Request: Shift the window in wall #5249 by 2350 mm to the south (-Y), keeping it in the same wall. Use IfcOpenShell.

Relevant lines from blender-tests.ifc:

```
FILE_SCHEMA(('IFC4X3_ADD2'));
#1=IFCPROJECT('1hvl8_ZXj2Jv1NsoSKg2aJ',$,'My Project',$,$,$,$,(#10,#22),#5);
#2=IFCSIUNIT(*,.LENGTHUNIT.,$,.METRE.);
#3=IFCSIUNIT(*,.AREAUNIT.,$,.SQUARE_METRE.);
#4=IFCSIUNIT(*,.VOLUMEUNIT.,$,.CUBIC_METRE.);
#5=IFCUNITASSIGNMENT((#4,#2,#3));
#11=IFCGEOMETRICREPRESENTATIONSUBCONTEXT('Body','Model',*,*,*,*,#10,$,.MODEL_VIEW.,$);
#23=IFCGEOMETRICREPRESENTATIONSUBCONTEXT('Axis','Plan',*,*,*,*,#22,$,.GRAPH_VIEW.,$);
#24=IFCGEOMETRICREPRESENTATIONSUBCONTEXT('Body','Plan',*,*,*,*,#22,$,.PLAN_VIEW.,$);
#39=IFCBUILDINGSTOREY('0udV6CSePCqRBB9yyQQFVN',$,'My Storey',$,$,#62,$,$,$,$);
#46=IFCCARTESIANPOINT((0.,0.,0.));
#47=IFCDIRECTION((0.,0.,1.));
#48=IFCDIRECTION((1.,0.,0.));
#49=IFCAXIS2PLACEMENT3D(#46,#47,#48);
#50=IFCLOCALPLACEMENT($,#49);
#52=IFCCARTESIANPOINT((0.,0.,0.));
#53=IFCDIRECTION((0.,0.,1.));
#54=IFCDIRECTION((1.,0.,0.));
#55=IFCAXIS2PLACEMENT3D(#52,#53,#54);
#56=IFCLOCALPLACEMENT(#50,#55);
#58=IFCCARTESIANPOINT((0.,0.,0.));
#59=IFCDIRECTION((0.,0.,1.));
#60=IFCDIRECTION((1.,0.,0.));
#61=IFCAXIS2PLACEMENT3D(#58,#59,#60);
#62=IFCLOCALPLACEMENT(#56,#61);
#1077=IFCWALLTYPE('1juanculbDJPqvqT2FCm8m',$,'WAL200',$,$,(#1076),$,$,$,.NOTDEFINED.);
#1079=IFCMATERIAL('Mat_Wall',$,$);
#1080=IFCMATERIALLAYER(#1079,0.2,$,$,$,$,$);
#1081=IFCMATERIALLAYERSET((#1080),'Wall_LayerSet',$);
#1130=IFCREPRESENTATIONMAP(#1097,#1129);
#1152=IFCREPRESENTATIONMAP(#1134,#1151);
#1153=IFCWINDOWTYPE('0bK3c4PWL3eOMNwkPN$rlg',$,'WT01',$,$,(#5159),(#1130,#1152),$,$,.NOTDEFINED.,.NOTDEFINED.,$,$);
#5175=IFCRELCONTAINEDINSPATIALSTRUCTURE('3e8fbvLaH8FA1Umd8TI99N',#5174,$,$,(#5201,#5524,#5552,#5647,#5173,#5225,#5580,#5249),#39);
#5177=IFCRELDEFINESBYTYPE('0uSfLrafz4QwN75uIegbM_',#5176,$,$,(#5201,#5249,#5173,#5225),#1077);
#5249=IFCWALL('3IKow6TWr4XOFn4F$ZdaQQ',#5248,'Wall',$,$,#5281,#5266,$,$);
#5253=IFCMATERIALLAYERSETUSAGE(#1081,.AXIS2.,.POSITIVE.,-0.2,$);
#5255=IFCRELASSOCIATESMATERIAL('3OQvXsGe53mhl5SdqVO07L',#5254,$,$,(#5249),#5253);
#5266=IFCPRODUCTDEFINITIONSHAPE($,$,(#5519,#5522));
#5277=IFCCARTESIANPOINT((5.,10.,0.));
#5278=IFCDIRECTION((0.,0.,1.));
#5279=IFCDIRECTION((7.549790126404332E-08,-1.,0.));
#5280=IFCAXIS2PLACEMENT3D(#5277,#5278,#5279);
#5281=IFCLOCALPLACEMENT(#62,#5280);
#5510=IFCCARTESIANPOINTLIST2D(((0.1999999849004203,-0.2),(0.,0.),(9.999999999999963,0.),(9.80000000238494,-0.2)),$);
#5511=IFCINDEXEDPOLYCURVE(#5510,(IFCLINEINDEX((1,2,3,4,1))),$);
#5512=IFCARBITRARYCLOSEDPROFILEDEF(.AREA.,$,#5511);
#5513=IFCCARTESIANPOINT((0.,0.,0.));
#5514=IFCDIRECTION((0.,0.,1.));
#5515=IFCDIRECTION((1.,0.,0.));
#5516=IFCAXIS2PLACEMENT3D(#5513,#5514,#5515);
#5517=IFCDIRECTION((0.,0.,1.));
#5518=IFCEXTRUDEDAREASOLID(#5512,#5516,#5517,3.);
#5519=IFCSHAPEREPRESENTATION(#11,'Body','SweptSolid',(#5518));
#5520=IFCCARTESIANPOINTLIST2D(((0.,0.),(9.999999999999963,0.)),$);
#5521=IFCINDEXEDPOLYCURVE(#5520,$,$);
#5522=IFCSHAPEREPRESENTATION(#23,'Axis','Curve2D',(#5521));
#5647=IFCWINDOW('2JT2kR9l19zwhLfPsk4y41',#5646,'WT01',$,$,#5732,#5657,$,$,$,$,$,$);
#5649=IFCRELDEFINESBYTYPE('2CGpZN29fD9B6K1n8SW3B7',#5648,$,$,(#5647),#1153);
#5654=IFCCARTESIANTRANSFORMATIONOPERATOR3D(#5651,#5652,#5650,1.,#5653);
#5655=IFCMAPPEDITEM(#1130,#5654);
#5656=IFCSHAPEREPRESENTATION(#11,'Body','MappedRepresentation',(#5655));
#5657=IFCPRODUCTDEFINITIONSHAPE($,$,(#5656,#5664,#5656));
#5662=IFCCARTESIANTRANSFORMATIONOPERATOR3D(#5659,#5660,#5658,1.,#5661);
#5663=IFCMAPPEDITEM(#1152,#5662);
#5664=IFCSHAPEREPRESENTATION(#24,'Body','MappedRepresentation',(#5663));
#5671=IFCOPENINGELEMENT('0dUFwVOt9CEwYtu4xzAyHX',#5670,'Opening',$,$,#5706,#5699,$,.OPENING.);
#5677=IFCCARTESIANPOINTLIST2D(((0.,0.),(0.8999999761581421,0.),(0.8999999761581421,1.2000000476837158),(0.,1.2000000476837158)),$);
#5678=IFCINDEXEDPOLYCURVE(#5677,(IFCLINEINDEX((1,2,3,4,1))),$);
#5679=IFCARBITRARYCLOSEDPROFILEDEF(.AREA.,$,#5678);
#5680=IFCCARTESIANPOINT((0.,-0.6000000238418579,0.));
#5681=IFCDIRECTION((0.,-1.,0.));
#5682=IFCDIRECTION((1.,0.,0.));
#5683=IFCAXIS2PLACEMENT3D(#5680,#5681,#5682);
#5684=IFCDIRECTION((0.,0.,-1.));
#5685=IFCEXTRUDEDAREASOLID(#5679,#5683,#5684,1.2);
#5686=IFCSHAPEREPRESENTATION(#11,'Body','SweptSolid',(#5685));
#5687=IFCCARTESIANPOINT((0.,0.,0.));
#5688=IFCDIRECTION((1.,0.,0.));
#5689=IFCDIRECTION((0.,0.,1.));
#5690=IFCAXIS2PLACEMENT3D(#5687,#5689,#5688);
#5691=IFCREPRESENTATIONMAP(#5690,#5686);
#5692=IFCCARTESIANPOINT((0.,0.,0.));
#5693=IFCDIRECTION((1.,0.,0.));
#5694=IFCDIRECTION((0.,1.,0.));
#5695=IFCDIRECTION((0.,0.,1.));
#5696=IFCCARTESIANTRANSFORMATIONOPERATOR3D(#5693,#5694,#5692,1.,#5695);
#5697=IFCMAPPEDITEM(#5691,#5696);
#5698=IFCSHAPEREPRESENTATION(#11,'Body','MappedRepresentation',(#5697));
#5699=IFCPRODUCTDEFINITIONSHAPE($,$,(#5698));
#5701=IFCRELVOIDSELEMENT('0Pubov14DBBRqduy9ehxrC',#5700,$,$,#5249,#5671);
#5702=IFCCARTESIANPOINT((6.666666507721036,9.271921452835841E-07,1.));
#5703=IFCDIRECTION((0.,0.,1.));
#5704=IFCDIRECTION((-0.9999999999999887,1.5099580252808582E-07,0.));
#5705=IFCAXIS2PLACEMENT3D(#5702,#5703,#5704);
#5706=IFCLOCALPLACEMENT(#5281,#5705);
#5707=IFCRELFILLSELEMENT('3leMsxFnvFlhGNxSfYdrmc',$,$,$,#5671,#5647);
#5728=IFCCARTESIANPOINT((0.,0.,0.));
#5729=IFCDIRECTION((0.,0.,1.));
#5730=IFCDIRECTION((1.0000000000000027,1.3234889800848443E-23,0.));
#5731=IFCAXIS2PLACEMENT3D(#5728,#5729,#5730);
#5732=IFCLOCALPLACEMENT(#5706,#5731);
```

```python
import ifcopenshell
import ifcopenshell.api.geometry
import ifcopenshell.util.placement

model = ifcopenshell.open("blender-tests.ifc")

window = model.by_id(5647)
opening = window.FillsVoids[0].RelatingOpeningElement
wall = opening.VoidsElements[0].RelatingBuildingElement

wall_matrix = ifcopenshell.util.placement.get_local_placement(wall.ObjectPlacement)
shift = wall_matrix[:3, 0] * 2.35
before = ifcopenshell.util.placement.get_local_placement(window.ObjectPlacement)[:3, 3].copy()

# The window is placed relative to its opening, so it follows when the opening moves.
matrix = ifcopenshell.util.placement.get_local_placement(opening.ObjectPlacement)
matrix[:3, 3] += shift
ifcopenshell.api.geometry.edit_object_placement(
    model, product=opening, matrix=matrix, is_si=False, should_transform_children=True
)

after = ifcopenshell.util.placement.get_local_placement(window.ObjectPlacement)[:3, 3]
print("window moved by", (after - before).round(3) + 0.0)

model.write("blender-tests_updated.ifc")
```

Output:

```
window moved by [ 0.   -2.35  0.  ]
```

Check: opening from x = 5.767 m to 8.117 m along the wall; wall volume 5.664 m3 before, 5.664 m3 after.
